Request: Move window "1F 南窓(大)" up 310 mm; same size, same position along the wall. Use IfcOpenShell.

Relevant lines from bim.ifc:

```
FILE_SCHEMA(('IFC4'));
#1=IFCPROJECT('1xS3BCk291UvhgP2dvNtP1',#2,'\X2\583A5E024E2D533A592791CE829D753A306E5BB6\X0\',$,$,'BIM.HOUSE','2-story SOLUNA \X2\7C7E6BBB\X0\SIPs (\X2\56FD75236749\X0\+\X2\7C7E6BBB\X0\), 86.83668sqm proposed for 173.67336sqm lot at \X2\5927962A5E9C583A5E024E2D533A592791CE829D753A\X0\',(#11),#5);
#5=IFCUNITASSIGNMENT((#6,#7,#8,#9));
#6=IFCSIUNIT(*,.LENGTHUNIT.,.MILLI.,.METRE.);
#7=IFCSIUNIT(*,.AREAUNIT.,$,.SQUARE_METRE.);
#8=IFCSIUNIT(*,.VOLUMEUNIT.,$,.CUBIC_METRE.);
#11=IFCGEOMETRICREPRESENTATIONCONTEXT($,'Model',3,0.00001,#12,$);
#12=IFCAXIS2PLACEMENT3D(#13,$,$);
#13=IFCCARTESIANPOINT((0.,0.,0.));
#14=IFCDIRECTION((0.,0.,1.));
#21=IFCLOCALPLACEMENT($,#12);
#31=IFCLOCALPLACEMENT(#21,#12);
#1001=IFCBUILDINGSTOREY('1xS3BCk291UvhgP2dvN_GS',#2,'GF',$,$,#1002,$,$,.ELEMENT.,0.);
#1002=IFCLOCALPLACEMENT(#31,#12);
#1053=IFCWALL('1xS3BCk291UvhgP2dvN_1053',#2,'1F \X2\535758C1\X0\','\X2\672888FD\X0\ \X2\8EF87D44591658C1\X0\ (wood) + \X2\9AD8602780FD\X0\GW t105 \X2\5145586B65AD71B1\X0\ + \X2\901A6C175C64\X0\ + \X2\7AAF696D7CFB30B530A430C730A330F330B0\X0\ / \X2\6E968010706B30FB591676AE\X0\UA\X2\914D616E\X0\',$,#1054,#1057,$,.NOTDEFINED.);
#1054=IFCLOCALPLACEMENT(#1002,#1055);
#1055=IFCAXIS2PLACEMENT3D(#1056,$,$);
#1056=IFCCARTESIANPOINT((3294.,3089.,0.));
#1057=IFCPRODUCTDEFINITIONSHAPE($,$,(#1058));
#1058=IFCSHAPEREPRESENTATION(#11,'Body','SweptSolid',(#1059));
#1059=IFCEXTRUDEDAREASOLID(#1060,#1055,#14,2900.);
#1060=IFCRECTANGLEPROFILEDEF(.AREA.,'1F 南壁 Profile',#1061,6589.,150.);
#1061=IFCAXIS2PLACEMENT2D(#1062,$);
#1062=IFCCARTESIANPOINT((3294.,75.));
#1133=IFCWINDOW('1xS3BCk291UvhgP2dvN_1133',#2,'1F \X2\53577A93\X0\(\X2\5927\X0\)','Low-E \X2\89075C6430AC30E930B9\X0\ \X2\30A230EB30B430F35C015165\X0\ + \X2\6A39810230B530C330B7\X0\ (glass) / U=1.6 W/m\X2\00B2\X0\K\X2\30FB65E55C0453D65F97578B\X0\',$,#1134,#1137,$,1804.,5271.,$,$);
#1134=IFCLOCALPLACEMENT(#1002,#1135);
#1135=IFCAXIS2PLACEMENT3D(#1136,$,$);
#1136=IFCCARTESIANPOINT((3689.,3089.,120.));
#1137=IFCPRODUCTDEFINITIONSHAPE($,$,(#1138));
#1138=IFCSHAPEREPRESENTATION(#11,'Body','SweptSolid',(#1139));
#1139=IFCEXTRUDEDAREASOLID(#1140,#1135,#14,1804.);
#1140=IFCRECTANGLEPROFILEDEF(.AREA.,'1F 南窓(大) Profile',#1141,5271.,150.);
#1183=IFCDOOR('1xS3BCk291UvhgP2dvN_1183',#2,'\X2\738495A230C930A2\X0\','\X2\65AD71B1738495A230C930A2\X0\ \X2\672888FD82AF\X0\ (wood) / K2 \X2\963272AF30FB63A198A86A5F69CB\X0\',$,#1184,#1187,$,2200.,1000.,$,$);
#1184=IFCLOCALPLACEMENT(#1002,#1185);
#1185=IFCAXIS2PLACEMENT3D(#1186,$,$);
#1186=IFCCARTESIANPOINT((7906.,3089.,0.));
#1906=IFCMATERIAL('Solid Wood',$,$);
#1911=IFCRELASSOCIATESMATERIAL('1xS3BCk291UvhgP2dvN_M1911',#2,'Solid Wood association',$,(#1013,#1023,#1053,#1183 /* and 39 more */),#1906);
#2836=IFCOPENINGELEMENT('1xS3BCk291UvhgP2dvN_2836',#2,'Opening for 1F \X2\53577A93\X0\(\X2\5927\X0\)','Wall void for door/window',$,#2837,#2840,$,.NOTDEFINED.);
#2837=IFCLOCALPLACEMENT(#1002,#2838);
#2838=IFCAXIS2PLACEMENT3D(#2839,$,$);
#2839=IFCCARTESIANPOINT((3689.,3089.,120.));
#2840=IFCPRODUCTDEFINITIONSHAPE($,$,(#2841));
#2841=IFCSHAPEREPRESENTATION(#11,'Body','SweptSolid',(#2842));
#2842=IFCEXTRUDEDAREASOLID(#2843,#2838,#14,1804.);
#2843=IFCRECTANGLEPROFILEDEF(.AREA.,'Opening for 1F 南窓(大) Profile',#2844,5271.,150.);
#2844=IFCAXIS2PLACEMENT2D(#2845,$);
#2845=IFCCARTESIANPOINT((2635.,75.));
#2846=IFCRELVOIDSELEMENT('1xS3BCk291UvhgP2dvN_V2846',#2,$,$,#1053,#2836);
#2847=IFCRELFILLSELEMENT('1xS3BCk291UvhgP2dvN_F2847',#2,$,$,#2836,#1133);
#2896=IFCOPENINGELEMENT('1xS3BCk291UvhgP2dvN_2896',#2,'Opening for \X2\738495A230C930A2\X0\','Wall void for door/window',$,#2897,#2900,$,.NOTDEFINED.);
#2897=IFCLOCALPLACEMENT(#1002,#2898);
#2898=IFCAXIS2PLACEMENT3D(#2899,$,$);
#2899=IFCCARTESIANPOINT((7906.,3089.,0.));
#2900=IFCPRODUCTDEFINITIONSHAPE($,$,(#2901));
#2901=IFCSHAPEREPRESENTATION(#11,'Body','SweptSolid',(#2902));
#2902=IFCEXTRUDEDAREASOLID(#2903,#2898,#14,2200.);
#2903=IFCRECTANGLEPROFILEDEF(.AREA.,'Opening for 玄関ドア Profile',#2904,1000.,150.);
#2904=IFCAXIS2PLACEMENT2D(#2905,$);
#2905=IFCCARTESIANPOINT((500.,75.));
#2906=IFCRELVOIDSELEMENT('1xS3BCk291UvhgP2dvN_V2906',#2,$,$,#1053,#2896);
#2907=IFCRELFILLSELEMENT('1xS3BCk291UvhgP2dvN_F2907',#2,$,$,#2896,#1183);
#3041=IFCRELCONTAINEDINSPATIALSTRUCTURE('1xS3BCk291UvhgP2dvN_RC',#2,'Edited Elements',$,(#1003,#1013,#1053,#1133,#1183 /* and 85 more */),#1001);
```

```python
import numpy as np
import ifcopenshell
import ifcopenshell.api.geometry
import ifcopenshell.util.placement
import ifcopenshell.util.unit

model = ifcopenshell.open("bim.ifc")
unit_scale = ifcopenshell.util.unit.calculate_unit_scale(model)

window = model.by_guid("1xS3BCk291UvhgP2dvN_1133")
opening = window.FillsVoids[0].RelatingOpeningElement
dz = 0.31 / unit_scale

shift = np.array([0.0, 0.0, dz])
# The window is not placed relative to its opening, so move both.
for product in (opening, window):
    matrix = ifcopenshell.util.placement.get_local_placement(product.ObjectPlacement)
    matrix[:3, 3] += shift
    ifcopenshell.api.geometry.edit_object_placement(model, product=product, matrix=matrix, is_si=False)

print(f"moved by {dz * unit_scale:+.3f} m")

model.write("bim_v2.ifc")
```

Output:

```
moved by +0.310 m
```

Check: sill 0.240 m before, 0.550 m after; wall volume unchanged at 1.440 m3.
